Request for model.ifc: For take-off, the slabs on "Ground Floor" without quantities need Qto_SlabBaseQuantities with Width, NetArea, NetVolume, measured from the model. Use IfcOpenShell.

First a look at what the model holds.

```python
import ifcopenshell
import ifcopenshell.util.element
import ifcopenshell.util.unit

model = ifcopenshell.open("model.ifc")
print(model.schema)
for unit_type in ("LENGTHUNIT", "AREAUNIT", "VOLUMEUNIT"):
    print(unit_type, ifcopenshell.util.unit.calculate_unit_scale(model, unit_type))
storey = next(s for s in model.by_type("IfcBuildingStorey") if s.Name == "Ground Floor")
slabs = [e for e in ifcopenshell.util.element.get_decomposition(storey) if e.is_a("IfcSlab")]
for e in sorted(slabs, key=lambda e: e.id()):
    print(e.id(), e.is_a(), e.Name, list(ifcopenshell.util.element.get_psets(e, qtos_only=True)), sep=" | ")
```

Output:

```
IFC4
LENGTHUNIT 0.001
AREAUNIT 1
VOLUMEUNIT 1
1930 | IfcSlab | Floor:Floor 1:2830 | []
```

```python
import ifcopenshell
import ifcopenshell.api.pset
import ifcopenshell.geom
import ifcopenshell.util.element
import ifcopenshell.util.shape
import ifcopenshell.util.unit

model = ifcopenshell.open("model.ifc")
unit_scale = ifcopenshell.util.unit.calculate_unit_scale(model)
area_scale = ifcopenshell.util.unit.calculate_unit_scale(model, "AREAUNIT")
volume_scale = ifcopenshell.util.unit.calculate_unit_scale(model, "VOLUMEUNIT")
settings = ifcopenshell.geom.settings()

storey = next(s for s in model.by_type("IfcBuildingStorey") if s.Name == "Ground Floor")
slabs = [e for e in ifcopenshell.util.element.get_decomposition(storey) if e.is_a("IfcSlab")]

for e in sorted(slabs, key=lambda e: e.id()):
    if ifcopenshell.util.element.get_psets(e, qtos_only=True, should_inherit=False):
        continue
    # Geometry comes back in metres, in the element's own axes.
    shape = ifcopenshell.geom.create_shape(settings, e)
    values = {
        "Width": ifcopenshell.util.shape.get_z(shape.geometry) / unit_scale,
        "NetArea": ifcopenshell.util.shape.get_footprint_area(shape.geometry) / area_scale,
        "NetVolume": ifcopenshell.util.shape.get_volume(shape.geometry) / volume_scale,
    }
    qto = ifcopenshell.api.pset.add_qto(model, product=e, name="Qto_SlabBaseQuantities")
    ifcopenshell.api.pset.edit_qto(model, qto=qto, properties=values)
    print(e.id(), {k: round(v, 3) for k, v in values.items()})

model.write("model_updated.ifc")
```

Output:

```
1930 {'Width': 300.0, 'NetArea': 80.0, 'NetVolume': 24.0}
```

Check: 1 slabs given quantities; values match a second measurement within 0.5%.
